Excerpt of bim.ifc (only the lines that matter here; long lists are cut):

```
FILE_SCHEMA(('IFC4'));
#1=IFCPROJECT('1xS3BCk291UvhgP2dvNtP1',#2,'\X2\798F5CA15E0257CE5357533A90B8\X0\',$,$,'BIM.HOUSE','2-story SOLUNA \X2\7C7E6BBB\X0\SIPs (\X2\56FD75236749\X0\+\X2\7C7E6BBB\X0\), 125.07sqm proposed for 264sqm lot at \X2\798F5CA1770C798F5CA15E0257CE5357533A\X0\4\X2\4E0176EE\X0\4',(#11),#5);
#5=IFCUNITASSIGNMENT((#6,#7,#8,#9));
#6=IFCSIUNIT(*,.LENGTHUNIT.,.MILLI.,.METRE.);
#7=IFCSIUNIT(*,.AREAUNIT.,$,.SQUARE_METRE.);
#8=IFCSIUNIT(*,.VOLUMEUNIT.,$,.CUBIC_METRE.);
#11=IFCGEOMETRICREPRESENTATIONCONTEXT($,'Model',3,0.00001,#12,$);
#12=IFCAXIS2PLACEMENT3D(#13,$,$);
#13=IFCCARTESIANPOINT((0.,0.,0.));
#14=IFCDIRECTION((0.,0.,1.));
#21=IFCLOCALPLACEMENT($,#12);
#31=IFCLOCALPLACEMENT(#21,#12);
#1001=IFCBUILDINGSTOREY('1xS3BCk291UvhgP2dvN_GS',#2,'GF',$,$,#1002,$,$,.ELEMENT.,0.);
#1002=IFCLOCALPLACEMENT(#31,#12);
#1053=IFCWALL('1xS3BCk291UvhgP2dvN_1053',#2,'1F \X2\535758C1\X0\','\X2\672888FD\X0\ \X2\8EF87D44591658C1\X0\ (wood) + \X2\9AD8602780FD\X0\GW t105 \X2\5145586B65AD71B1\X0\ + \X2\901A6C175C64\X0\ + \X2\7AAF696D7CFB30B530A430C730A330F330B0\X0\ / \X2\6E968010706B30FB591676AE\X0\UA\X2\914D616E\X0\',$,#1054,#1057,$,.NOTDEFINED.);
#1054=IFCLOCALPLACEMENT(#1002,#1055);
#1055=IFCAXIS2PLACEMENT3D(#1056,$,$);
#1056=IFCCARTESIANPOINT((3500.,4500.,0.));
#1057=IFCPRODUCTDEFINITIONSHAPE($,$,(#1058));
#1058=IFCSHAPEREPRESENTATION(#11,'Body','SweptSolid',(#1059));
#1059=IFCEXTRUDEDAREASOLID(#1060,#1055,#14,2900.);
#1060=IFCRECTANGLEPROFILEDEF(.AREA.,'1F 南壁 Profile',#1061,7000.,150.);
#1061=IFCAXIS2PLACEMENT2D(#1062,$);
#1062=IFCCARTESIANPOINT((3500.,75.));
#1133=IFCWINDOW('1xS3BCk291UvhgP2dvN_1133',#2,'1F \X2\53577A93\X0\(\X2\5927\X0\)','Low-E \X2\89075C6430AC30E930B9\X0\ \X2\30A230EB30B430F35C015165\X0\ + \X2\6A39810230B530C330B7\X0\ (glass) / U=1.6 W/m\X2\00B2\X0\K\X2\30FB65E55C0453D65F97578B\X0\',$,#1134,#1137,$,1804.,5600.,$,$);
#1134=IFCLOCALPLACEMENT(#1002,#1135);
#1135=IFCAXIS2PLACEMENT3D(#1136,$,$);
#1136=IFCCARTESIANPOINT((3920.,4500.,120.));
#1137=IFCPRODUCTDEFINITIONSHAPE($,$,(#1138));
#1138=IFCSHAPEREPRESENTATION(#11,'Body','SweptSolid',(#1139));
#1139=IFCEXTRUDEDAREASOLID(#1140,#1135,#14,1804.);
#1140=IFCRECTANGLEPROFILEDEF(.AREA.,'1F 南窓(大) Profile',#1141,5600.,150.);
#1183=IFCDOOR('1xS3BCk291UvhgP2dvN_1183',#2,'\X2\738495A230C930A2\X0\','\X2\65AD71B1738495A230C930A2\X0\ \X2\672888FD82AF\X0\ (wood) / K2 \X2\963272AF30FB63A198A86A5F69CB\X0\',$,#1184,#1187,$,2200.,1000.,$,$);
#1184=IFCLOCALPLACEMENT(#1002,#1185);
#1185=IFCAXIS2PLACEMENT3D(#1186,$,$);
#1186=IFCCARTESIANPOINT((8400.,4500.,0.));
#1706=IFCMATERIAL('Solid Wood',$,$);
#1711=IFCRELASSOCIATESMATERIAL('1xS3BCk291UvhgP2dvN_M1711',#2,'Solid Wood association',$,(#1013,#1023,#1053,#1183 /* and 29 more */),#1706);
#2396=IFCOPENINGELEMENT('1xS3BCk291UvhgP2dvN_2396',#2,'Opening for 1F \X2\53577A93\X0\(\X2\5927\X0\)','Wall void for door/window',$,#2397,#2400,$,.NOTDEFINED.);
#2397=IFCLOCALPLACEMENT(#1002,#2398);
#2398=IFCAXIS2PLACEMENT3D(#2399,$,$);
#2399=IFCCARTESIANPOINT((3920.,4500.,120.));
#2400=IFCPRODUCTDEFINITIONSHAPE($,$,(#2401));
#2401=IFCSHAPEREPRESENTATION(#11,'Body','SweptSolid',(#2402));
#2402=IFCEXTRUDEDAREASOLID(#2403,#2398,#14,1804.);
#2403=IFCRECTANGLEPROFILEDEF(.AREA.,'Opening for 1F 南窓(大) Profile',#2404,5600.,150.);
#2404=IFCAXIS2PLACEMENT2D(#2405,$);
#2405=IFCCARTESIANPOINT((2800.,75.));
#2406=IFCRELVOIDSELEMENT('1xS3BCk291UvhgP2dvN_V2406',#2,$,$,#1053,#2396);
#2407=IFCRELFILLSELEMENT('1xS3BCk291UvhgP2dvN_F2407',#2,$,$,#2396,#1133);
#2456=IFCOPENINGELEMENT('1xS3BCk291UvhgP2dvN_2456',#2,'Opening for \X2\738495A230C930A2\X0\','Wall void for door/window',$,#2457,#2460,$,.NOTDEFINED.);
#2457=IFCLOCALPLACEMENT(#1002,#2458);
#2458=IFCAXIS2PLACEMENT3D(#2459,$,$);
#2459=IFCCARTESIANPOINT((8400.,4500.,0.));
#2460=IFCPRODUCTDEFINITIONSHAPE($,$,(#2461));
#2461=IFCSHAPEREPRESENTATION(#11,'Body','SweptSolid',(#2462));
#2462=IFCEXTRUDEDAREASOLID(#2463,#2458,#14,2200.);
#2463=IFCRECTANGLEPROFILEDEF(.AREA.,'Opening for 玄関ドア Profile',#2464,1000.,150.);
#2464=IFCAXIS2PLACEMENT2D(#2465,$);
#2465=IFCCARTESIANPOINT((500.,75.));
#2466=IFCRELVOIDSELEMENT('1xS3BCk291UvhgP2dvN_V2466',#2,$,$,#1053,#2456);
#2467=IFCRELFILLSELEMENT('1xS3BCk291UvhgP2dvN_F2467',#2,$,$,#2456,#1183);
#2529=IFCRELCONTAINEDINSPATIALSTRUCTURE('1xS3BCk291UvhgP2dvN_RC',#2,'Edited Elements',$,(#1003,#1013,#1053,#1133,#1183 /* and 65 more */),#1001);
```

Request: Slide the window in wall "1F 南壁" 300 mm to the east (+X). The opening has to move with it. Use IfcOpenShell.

```python
import ifcopenshell
import ifcopenshell.api.geometry
import ifcopenshell.util.placement

model = ifcopenshell.open("bim.ifc")

window = model.by_id(1133)
opening = window.FillsVoids[0].RelatingOpeningElement
wall = opening.VoidsElements[0].RelatingBuildingElement

wall_matrix = ifcopenshell.util.placement.get_local_placement(wall.ObjectPlacement)
shift = wall_matrix[:3, 0] * 300.0
before = ifcopenshell.util.placement.get_local_placement(window.ObjectPlacement)[:3, 3].copy()

# The window is not placed relative to its opening, so move both.
for product in (opening, window):
    matrix = ifcopenshell.util.placement.get_local_placement(product.ObjectPlacement)
    matrix[:3, 3] += shift
    ifcopenshell.api.geometry.edit_object_placement(model, product=product, matrix=matrix, is_si=False)

after = ifcopenshell.util.placement.get_local_placement(window.ObjectPlacement)[:3, 3]
print("window moved by", (after - before).round(3) + 0.0)

model.write("bim_updated.ifc")
```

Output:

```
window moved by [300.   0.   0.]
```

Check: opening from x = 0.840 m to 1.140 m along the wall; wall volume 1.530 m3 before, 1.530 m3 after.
